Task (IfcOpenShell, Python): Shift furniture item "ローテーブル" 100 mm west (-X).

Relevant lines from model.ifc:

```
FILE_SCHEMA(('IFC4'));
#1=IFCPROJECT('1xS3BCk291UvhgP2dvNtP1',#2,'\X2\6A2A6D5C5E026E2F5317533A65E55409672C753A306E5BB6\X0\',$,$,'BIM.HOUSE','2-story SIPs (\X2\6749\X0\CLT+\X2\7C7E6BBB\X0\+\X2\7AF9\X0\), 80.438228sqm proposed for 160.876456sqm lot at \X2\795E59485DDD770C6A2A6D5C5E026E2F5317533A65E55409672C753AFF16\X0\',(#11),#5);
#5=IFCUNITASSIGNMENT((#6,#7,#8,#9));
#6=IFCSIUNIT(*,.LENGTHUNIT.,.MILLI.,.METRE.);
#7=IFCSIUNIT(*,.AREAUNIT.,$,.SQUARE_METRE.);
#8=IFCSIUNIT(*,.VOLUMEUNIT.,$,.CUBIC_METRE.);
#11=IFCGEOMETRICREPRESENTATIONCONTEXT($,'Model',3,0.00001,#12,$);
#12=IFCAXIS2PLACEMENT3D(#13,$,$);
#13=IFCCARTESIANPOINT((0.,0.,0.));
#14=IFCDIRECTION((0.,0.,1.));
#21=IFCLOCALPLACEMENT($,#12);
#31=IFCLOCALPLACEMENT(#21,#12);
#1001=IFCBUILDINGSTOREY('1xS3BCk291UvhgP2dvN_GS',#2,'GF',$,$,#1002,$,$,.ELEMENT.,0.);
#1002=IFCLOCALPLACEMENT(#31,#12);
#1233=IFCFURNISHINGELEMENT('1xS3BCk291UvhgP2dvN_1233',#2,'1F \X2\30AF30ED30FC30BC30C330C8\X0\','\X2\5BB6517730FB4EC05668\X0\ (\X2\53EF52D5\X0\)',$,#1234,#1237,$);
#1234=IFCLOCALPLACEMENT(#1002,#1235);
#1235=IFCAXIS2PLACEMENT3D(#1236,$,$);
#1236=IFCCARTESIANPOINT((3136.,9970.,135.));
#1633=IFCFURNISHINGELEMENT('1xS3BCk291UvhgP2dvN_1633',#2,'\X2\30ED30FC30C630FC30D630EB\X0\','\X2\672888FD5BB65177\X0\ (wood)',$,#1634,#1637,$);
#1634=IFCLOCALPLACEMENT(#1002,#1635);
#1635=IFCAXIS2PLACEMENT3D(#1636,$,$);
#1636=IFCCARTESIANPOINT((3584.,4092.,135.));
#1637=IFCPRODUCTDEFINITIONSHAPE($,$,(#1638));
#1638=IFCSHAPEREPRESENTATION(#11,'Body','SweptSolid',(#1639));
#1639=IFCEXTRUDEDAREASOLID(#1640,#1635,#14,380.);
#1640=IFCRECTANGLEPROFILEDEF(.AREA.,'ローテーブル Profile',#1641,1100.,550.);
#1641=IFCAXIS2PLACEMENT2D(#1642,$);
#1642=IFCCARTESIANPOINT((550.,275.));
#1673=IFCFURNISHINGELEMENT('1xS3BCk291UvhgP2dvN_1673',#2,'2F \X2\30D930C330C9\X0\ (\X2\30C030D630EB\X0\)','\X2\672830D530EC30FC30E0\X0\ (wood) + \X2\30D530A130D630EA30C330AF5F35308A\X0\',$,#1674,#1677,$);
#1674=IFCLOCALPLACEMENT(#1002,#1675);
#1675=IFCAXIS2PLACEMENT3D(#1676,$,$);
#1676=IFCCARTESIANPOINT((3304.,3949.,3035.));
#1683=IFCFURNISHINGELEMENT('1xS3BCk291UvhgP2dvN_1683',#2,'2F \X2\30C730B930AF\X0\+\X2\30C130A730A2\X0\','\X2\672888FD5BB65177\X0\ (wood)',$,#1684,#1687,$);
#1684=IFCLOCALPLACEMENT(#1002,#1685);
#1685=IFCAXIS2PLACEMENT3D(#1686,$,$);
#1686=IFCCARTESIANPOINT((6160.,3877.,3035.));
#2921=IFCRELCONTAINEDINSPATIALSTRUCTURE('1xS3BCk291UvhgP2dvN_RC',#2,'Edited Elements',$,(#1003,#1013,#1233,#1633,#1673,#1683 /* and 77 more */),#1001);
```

```python
import ifcopenshell
import ifcopenshell.api.geometry
import ifcopenshell.util.placement
import ifcopenshell.util.unit

model = ifcopenshell.open("model.ifc")
unit_scale = ifcopenshell.util.unit.calculate_unit_scale(model)

item = model.by_id(1633)
matrix = ifcopenshell.util.placement.get_local_placement(item.ObjectPlacement)
matrix[0, 3] -= 0.1 / unit_scale
ifcopenshell.api.geometry.edit_object_placement(model, product=item, matrix=matrix, is_si=False)

print(ifcopenshell.util.placement.get_local_placement(item.ObjectPlacement).round(3) + 0.0)

model.write("model_rev.ifc")
```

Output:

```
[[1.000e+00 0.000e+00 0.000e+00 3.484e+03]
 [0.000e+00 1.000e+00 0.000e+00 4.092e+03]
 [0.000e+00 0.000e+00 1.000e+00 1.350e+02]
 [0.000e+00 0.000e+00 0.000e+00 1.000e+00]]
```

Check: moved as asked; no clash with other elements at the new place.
